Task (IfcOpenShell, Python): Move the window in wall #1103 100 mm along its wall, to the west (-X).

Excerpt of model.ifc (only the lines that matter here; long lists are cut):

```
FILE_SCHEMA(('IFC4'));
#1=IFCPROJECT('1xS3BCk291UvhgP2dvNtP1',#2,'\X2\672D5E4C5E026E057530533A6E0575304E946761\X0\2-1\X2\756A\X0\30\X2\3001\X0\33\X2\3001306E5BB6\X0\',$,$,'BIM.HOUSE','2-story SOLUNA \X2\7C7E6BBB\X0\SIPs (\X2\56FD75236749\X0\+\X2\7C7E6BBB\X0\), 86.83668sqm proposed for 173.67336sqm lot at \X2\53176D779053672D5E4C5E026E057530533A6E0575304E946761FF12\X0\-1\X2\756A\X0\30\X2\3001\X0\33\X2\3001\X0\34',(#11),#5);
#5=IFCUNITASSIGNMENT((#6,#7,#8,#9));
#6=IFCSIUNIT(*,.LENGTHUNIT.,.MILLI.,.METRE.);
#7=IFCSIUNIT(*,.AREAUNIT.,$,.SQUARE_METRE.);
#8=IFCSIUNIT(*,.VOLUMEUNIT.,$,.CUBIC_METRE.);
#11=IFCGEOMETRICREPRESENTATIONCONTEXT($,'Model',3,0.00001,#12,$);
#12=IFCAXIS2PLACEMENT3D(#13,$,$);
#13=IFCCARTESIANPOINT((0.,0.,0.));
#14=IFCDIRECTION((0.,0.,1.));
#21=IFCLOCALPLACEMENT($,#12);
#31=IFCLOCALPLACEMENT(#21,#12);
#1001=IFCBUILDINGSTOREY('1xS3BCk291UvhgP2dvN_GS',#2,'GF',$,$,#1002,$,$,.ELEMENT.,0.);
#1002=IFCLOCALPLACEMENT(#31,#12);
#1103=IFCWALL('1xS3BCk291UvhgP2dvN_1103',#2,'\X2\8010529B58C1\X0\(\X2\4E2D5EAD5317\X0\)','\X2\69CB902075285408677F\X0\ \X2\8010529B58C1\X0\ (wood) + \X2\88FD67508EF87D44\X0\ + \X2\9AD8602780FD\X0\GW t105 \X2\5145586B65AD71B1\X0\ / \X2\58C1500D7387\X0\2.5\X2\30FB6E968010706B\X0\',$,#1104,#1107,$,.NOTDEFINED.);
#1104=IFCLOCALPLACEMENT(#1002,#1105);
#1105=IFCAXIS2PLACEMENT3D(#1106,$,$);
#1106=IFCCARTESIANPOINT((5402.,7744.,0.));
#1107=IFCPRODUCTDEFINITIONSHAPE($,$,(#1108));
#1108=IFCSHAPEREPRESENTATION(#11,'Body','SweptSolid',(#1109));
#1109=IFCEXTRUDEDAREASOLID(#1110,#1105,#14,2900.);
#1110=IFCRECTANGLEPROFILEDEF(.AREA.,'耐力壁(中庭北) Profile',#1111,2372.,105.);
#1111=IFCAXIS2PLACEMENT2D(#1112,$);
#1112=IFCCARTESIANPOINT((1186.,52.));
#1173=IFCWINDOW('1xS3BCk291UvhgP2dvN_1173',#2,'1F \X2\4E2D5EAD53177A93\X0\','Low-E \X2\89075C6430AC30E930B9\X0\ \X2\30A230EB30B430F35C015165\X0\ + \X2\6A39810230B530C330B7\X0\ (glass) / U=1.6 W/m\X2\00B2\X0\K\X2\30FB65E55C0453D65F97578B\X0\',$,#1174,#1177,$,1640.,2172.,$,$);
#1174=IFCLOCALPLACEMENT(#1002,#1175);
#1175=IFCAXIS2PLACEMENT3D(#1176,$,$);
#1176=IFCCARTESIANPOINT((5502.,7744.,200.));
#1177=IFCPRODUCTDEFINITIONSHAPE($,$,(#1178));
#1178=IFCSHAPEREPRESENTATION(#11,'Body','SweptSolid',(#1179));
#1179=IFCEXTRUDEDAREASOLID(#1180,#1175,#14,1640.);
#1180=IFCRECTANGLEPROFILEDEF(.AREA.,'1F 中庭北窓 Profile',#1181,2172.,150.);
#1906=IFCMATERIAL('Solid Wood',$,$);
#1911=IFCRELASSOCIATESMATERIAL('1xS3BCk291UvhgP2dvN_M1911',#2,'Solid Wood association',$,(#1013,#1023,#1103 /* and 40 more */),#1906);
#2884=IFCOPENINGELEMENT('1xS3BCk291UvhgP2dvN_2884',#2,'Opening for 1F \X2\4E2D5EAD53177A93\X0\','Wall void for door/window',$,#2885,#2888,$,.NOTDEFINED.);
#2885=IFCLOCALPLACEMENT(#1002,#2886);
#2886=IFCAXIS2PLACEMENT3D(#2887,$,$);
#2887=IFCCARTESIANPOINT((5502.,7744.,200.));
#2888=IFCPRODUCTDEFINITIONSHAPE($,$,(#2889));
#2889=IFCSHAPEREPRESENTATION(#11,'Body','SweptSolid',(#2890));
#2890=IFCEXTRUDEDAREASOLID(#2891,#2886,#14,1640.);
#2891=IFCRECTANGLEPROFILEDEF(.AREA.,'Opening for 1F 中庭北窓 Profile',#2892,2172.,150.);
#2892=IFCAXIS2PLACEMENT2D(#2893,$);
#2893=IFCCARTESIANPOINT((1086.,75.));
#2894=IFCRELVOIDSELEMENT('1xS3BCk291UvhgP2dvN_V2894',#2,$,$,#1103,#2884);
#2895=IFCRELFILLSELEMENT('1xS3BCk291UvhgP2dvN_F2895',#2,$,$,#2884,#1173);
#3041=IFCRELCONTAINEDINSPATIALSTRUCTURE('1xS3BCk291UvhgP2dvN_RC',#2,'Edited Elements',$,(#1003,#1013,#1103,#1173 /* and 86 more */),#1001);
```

```python
import ifcopenshell
import ifcopenshell.api.geometry
import ifcopenshell.util.placement
import ifcopenshell.util.unit

model = ifcopenshell.open("model.ifc")
unit_scale = ifcopenshell.util.unit.calculate_unit_scale(model)

window = model.by_id(1173)
opening = window.FillsVoids[0].RelatingOpeningElement
wall = opening.VoidsElements[0].RelatingBuildingElement

wall_matrix = ifcopenshell.util.placement.get_local_placement(wall.ObjectPlacement)
shift = wall_matrix[:3, 0] * -0.1 / unit_scale
before = ifcopenshell.util.placement.get_local_placement(window.ObjectPlacement)[:3, 3].copy()

# The window is not placed relative to its opening, so move both.
for product in (opening, window):
    matrix = ifcopenshell.util.placement.get_local_placement(product.ObjectPlacement)
    matrix[:3, 3] += shift
    ifcopenshell.api.geometry.edit_object_placement(model, product=product, matrix=matrix, is_si=False)

after = ifcopenshell.util.placement.get_local_placement(window.ObjectPlacement)[:3, 3]
print("window moved by", (after - before).round(3) + 0.0)

model.write("model_updated.ifc")
```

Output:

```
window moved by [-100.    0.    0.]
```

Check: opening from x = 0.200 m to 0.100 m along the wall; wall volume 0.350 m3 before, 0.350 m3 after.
